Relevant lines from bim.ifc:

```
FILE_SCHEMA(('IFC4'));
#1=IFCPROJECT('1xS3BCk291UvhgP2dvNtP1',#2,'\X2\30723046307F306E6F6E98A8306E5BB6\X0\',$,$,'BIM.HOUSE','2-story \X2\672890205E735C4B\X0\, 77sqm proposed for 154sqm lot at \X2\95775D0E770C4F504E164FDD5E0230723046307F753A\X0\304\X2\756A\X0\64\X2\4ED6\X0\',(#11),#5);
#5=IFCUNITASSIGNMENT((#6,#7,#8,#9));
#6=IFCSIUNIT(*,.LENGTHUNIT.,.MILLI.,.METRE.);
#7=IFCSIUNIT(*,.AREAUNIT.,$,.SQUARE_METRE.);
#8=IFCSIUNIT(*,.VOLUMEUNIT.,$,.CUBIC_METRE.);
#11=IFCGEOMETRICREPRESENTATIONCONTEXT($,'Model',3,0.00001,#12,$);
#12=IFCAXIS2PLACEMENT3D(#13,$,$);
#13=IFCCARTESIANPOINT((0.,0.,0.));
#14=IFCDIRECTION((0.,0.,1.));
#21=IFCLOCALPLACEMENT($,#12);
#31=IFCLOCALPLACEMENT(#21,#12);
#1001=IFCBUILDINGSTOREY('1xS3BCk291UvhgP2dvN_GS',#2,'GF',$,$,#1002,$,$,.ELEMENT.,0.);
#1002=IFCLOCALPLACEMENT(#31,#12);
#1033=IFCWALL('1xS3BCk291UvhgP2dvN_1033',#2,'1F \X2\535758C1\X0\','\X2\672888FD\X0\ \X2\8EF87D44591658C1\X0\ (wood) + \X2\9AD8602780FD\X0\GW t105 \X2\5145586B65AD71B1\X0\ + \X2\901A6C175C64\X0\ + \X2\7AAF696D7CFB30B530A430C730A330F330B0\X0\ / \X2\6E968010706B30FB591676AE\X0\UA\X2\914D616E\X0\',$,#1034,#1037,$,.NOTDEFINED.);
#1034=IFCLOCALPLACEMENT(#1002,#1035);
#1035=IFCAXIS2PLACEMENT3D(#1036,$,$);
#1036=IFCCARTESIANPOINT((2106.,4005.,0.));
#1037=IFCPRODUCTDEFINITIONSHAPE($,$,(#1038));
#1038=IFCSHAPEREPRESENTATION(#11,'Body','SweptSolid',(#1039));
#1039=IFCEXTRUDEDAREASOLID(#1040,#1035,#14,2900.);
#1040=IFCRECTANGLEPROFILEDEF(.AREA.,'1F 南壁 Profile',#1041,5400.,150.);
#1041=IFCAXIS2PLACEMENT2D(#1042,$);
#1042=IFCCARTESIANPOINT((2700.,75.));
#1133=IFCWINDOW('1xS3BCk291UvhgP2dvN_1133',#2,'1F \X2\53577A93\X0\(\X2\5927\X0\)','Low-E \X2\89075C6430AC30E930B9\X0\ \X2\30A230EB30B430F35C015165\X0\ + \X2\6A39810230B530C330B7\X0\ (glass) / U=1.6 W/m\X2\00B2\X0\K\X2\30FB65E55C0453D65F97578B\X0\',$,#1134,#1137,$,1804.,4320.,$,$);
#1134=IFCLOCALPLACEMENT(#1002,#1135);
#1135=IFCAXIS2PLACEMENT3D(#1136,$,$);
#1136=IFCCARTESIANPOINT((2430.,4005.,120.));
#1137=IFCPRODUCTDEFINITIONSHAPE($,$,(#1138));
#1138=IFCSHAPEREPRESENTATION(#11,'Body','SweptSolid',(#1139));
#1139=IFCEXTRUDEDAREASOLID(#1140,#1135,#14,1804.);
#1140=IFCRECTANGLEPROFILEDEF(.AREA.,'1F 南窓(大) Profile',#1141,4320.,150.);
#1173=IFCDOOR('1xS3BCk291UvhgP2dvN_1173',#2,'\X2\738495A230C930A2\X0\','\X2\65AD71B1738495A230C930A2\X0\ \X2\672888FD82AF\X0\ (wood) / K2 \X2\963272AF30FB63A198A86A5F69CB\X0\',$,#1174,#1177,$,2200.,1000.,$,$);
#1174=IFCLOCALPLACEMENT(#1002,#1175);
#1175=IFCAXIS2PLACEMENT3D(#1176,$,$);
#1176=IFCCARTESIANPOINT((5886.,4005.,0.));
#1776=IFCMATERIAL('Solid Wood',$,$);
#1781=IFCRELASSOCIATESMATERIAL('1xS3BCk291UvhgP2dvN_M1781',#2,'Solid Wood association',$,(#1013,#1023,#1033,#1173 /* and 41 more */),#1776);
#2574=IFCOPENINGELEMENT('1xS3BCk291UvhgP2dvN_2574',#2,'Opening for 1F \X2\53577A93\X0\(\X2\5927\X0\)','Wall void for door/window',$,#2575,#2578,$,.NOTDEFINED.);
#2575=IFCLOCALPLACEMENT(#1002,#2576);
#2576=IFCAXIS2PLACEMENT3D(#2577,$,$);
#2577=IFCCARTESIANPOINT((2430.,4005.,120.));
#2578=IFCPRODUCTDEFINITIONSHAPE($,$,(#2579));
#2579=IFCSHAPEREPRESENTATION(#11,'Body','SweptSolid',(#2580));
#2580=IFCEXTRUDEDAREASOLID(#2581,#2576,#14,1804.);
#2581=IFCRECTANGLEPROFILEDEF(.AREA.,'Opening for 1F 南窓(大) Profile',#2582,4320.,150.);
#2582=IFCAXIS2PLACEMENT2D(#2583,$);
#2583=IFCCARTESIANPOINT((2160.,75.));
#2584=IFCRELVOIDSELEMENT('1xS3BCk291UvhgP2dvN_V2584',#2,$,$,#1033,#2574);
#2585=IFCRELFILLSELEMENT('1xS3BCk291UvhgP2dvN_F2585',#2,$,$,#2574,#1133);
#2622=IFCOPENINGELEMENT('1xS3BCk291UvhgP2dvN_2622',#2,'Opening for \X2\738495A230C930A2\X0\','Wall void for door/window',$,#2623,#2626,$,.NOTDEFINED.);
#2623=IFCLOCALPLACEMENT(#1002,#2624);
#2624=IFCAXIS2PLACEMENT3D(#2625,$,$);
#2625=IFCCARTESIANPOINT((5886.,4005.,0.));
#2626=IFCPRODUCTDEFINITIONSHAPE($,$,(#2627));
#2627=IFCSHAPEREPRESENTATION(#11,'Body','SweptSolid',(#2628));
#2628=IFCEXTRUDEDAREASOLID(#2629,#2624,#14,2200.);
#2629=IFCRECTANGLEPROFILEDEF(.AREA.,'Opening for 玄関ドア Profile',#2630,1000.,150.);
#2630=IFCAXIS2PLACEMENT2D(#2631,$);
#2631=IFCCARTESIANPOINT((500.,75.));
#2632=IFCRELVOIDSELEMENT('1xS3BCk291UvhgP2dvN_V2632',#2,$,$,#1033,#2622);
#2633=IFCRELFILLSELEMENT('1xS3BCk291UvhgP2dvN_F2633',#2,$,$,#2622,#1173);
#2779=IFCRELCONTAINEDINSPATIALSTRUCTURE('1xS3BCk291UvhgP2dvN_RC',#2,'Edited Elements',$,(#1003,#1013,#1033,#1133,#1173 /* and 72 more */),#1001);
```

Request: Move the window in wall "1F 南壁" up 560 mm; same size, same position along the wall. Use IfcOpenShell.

```python
import numpy as np
import ifcopenshell
import ifcopenshell.api.geometry
import ifcopenshell.util.placement
import ifcopenshell.util.unit

model = ifcopenshell.open("bim.ifc")
unit_scale = ifcopenshell.util.unit.calculate_unit_scale(model)

window = model.by_id(1133)
opening = window.FillsVoids[0].RelatingOpeningElement
dz = 0.56 / unit_scale

shift = np.array([0.0, 0.0, dz])
# The window is not placed relative to its opening, so move both.
for product in (opening, window):
    matrix = ifcopenshell.util.placement.get_local_placement(product.ObjectPlacement)
    matrix[:3, 3] += shift
    ifcopenshell.api.geometry.edit_object_placement(model, product=product, matrix=matrix, is_si=False)

print(f"moved by {dz * unit_scale:+.3f} m")

model.write("bim_edited.ifc")
```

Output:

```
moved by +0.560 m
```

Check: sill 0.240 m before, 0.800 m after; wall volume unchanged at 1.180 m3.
